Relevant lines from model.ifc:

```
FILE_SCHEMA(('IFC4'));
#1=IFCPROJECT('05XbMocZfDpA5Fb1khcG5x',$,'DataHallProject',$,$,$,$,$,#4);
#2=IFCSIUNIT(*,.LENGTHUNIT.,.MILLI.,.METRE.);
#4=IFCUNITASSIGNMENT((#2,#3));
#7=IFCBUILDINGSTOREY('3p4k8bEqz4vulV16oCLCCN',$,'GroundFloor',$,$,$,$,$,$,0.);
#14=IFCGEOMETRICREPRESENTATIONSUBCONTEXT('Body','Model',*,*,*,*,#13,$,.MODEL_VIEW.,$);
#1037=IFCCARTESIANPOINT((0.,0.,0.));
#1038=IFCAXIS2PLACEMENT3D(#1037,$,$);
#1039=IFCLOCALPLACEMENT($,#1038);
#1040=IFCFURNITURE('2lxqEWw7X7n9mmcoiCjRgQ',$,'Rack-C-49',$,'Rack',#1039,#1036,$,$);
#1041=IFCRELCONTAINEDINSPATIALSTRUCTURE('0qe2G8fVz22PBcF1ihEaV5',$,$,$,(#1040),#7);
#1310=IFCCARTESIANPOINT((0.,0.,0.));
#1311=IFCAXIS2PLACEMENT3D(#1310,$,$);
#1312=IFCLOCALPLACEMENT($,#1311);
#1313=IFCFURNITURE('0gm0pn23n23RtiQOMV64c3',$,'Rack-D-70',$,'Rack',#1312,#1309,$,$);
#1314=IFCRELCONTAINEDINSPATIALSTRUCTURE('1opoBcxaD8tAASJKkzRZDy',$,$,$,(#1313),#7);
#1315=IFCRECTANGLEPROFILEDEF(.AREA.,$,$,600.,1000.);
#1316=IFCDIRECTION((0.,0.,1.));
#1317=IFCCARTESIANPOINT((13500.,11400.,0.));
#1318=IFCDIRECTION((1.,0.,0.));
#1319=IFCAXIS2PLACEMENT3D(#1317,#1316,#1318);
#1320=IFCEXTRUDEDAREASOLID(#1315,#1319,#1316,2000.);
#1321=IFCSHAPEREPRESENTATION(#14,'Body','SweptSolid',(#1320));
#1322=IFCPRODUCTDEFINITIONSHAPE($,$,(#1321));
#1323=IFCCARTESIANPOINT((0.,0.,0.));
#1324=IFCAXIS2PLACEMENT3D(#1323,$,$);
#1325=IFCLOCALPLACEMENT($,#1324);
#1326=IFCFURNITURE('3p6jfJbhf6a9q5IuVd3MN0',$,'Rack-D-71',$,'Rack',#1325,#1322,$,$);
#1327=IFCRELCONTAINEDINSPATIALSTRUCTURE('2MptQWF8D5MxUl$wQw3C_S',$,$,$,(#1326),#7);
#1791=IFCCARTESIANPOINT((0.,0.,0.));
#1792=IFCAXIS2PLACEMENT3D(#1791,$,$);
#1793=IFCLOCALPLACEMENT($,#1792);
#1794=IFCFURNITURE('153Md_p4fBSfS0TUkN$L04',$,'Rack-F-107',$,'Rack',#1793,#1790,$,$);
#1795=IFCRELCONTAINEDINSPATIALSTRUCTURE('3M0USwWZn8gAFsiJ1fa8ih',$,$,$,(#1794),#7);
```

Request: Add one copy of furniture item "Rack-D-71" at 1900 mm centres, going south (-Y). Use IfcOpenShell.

```python
import numpy as np
import ifcopenshell
import ifcopenshell.api.geometry
import ifcopenshell.api.root
import ifcopenshell.util.element
import ifcopenshell.util.placement

model = ifcopenshell.open("model.ifc")

source = model.by_id(1326)
base = ifcopenshell.util.placement.get_local_placement(source.ObjectPlacement)
step = np.array([0.0, -1.0, 0.0]) * 1900.0

for i in range(1, 2):
    copy = ifcopenshell.api.root.copy_class(model, product=source)
    copy.Representation = ifcopenshell.util.element.copy_deep(
        model, source.Representation, exclude=["IfcGeometricRepresentationContext", "IfcRepresentationMap"]
    )
    matrix = base.copy()
    matrix[:3, 3] += i * step
    print("added at", matrix[:3, 3].round(3) + 0.0)
    ifcopenshell.api.geometry.edit_object_placement(model, product=copy, matrix=matrix, is_si=False)

model.write("model_rev.ifc")
```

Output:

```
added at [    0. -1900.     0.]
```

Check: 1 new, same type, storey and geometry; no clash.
